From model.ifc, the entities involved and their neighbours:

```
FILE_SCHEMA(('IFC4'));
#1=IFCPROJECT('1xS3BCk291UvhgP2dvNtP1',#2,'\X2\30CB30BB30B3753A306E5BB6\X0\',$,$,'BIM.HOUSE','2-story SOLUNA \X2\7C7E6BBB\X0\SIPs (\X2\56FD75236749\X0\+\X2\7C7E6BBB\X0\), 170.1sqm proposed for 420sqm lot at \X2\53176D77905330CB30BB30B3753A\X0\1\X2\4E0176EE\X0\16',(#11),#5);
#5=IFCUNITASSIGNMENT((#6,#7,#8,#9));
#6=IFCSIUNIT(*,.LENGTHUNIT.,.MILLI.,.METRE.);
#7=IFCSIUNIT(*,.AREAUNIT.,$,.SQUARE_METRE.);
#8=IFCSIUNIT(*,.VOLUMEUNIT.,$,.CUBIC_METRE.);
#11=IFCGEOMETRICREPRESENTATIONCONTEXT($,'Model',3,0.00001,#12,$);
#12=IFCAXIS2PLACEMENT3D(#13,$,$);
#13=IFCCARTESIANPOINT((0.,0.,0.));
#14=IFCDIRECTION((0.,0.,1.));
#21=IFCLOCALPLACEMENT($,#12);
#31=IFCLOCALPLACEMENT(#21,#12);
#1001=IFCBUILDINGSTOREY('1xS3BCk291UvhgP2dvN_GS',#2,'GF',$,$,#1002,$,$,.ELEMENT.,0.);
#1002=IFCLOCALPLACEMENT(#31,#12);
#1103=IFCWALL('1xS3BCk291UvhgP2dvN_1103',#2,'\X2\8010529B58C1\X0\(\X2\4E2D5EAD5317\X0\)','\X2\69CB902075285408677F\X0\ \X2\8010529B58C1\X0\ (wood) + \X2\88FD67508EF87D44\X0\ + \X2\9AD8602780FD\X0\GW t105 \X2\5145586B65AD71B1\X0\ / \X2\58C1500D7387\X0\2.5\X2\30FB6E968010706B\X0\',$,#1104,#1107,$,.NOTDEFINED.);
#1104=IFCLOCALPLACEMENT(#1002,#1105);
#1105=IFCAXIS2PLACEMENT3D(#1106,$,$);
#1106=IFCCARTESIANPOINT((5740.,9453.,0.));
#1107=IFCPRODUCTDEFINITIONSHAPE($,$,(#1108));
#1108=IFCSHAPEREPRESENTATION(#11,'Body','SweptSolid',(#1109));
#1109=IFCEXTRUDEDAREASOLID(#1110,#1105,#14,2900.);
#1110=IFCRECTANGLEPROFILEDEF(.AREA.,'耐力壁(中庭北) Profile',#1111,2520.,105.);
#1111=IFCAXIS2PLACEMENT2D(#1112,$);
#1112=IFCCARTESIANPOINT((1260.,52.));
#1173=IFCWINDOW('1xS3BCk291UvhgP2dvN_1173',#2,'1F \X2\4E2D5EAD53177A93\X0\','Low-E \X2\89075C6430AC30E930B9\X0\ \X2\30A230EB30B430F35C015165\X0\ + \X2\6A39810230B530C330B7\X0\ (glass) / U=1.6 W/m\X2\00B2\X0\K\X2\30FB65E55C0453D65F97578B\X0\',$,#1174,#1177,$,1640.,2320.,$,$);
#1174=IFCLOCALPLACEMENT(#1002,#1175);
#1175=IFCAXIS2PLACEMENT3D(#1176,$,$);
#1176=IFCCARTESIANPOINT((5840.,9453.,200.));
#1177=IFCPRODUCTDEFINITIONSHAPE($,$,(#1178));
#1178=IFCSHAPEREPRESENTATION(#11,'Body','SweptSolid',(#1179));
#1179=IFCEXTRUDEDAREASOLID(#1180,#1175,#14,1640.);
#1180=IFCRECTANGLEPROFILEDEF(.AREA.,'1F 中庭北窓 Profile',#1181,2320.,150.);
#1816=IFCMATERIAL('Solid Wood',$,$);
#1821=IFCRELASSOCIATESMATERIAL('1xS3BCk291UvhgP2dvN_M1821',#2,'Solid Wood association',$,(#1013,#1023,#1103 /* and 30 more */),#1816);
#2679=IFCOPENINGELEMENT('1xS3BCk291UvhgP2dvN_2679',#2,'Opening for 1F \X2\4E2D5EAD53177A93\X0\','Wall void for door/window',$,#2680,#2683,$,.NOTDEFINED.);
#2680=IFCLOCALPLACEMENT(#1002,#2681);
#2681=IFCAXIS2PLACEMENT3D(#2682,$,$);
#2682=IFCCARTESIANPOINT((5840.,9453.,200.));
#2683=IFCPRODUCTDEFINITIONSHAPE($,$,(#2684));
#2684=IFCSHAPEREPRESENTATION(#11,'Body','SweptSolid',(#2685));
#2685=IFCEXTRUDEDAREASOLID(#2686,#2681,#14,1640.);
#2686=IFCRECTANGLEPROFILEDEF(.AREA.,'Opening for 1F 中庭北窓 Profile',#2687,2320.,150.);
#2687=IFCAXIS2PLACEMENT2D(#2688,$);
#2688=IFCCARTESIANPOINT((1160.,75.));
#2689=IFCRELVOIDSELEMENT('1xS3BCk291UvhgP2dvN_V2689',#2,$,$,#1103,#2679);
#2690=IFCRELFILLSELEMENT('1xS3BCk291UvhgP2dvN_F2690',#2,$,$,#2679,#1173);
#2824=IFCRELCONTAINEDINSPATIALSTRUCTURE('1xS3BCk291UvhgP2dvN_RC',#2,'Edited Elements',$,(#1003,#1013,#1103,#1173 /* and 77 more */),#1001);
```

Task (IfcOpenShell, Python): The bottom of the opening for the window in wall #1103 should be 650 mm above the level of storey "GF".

```python
import numpy as np
import ifcopenshell
import ifcopenshell.api.geometry
import ifcopenshell.geom
import ifcopenshell.util.element
import ifcopenshell.util.placement
import ifcopenshell.util.shape
import ifcopenshell.util.unit

model = ifcopenshell.open("model.ifc")
unit_scale = ifcopenshell.util.unit.calculate_unit_scale(model)

window = model.by_guid("1xS3BCk291UvhgP2dvN_1173")
opening = window.FillsVoids[0].RelatingOpeningElement
storey = ifcopenshell.util.element.get_container(window, ifc_class="IfcBuildingStorey")
level = ifcopenshell.util.placement.get_local_placement(storey.ObjectPlacement)[2, 3]

# The opening's origin need not be at the sill, so measure its lowest point.
shape = ifcopenshell.geom.create_shape(ifcopenshell.geom.settings(), opening)
bottom = ifcopenshell.util.shape.get_shape_bottom_elevation(shape, shape.geometry) / unit_scale
dz = level + 650.0 - bottom

shift = np.array([0.0, 0.0, dz])
# The window is not placed relative to its opening, so move both.
for product in (opening, window):
    matrix = ifcopenshell.util.placement.get_local_placement(product.ObjectPlacement)
    matrix[:3, 3] += shift
    ifcopenshell.api.geometry.edit_object_placement(model, product=product, matrix=matrix, is_si=False)

print(f"moved by {dz * unit_scale:+.3f} m")

model.write("model_rev.ifc")
```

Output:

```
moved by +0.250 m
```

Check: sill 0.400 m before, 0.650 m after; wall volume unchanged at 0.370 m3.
